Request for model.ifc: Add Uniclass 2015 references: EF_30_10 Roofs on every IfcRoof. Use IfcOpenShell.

First a look at what the model holds.

```python
import ifcopenshell

model = ifcopenshell.open("model.ifc")
print(model.schema)
print("classifications:", [c.Name for c in model.by_type("IfcClassification")])
for ifc_class in ("IfcDoor", "IfcRoof", "IfcStair", "IfcWall", "IfcWindow"):
    print(ifc_class, len(model.by_type(ifc_class)))
```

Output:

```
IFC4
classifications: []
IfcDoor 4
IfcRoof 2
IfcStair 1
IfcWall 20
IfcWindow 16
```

```python
import ifcopenshell
import ifcopenshell.api.classification

model = ifcopenshell.open("model.ifc")

system = ifcopenshell.api.classification.add_classification(model, classification="Uniclass 2015")

codes = {
    "IfcRoof": ("EF_30_10", "Roofs"),
}
for ifc_class, (code, name) in codes.items():
    products = model.by_type(ifc_class)
    ifcopenshell.api.classification.add_reference(
        model, products=products, classification=system, identification=code, name=name
    )
    print(code, len(products))

model.write("model_updated.ifc")
```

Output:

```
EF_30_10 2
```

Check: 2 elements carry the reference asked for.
